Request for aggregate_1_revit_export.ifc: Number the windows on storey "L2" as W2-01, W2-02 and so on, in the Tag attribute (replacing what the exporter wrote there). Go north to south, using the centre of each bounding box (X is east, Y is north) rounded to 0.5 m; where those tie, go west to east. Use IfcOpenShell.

First a look at what the model holds.

```python
import ifcopenshell
import ifcopenshell.util.element
import ifcopenshell.util.placement

model = ifcopenshell.open("aggregate_1_revit_export.ifc")
print(model.schema)
storey = next(s for s in model.by_type("IfcBuildingStorey") if s.Name == "L2")
windows = [e for e in ifcopenshell.util.element.get_decomposition(storey) if e.is_a("IfcWindow")]
for e in sorted(windows, key=lambda e: e.id()):
    origin = ifcopenshell.util.placement.get_local_placement(e.ObjectPlacement)[:3, 3]
    print(e.id(), e.Tag, e.Name, origin.round(2) + 0.0, sep=" | ")
```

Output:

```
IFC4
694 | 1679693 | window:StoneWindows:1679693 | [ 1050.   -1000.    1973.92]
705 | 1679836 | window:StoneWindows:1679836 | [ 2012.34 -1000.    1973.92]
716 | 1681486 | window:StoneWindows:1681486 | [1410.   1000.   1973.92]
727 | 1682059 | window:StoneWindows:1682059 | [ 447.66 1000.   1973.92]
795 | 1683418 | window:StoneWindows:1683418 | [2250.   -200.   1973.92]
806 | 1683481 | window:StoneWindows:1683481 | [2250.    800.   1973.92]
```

```python
import ifcopenshell
import ifcopenshell.geom
import ifcopenshell.util.element
import ifcopenshell.util.shape

model = ifcopenshell.open("aggregate_1_revit_export.ifc")
settings = ifcopenshell.geom.settings()
settings.set("use-world-coords", True)


def centre(element):
    shape = ifcopenshell.geom.create_shape(settings, element)
    return ifcopenshell.util.shape.get_bbox_centroid(shape.geometry)


storey = next(s for s in model.by_type("IfcBuildingStorey") if s.Name == "L2")
windows = [e for e in ifcopenshell.util.element.get_decomposition(storey) if e.is_a("IfcWindow")]

# Insertion points can sit at a corner or the storey origin, so sort by the geometry (in metres).
centres = {e: centre(e) for e in windows}
windows.sort(key=lambda e: (-round(centres[e][1] / 0.5), centres[e][0]))

for i, e in enumerate(windows, start=1):
    number = f"W2-{i:02d}"
    e.Tag = number
    print(e.id(), number)

model.write("aggregate_1_revit_export-out.ifc")
```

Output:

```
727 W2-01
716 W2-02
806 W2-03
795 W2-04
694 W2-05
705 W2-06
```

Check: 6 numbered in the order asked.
